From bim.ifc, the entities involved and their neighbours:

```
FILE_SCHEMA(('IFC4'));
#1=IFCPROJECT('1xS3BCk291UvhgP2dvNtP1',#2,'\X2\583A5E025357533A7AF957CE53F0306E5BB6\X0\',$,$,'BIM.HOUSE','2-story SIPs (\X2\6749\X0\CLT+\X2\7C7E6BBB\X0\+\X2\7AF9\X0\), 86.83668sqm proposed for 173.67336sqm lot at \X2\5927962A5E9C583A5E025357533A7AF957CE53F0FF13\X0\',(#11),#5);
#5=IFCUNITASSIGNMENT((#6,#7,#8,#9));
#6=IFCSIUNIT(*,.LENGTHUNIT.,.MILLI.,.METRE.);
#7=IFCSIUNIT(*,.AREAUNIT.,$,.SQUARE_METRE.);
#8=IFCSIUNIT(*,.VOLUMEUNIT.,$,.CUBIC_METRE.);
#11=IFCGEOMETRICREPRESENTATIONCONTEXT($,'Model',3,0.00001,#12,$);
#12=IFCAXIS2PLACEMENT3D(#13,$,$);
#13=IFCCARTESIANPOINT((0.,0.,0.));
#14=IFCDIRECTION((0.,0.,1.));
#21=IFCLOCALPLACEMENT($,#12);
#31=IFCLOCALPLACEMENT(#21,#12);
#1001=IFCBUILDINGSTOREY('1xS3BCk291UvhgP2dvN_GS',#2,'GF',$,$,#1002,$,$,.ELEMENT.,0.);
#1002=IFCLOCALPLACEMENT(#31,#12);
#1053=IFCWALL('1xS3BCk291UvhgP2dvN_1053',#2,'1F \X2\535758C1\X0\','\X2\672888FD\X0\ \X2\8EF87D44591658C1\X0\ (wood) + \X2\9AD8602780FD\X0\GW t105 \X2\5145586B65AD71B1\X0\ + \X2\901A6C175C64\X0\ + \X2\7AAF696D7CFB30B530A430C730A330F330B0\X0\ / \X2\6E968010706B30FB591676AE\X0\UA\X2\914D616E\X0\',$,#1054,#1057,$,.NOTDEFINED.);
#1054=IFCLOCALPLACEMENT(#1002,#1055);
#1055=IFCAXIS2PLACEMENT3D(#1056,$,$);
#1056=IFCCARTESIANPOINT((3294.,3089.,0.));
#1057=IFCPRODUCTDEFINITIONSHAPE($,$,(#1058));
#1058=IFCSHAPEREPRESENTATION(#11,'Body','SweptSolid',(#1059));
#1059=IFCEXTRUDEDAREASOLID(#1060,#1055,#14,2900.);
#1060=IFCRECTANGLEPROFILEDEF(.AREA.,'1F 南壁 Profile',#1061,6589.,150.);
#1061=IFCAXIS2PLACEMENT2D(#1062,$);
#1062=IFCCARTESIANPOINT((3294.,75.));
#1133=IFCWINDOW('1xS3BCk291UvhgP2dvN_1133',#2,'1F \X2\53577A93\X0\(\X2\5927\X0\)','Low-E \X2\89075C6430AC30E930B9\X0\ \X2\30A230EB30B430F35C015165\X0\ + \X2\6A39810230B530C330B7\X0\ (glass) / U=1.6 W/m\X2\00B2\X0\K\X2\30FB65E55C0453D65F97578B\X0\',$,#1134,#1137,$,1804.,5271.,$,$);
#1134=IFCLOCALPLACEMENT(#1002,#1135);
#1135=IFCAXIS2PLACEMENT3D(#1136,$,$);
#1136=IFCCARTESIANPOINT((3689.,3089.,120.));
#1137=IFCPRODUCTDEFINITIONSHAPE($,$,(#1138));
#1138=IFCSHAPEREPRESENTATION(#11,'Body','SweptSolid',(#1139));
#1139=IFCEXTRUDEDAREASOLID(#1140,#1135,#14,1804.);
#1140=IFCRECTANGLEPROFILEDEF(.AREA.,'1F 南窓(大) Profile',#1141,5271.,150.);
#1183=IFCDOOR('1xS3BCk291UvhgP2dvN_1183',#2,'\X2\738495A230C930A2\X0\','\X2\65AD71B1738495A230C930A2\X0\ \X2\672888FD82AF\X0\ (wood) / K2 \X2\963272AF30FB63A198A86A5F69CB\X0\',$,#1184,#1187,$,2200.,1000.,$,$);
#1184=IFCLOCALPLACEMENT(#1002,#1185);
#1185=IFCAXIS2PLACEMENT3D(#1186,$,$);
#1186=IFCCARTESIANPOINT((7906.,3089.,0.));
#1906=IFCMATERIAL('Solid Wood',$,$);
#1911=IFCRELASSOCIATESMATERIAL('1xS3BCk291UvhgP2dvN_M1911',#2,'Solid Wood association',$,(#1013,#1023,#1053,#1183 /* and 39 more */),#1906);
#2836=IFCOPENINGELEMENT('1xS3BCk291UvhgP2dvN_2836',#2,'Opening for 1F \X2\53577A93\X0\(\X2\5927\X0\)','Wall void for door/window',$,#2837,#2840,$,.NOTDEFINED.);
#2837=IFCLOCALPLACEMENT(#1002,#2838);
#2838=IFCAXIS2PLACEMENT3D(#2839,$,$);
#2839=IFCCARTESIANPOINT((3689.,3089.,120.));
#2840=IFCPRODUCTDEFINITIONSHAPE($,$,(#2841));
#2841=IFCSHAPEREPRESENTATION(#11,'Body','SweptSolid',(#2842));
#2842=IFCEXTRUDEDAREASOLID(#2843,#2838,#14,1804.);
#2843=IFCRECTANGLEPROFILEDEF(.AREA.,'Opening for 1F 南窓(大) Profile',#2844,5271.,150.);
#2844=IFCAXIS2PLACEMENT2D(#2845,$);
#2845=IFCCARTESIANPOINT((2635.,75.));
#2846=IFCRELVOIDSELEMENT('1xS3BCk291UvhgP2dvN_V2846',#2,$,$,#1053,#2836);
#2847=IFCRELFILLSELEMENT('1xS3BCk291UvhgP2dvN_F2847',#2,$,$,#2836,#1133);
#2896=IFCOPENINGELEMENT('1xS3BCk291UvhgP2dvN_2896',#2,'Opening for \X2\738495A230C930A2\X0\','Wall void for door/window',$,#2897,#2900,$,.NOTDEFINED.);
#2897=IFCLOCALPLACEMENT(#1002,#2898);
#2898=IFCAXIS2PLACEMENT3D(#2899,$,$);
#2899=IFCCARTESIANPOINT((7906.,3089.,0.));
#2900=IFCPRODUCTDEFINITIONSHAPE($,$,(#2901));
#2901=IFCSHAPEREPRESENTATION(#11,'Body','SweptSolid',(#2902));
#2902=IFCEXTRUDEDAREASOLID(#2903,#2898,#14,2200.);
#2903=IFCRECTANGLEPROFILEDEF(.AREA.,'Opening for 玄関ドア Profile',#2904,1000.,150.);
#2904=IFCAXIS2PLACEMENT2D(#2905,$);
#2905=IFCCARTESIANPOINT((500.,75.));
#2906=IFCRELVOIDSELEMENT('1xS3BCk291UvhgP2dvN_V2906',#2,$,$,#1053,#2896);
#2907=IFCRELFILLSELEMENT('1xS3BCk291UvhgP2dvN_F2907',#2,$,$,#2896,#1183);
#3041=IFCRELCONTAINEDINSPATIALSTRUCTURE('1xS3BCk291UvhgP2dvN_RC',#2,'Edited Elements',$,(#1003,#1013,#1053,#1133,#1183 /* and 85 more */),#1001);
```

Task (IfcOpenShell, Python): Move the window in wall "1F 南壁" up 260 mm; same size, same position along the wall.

```python
import numpy as np
import ifcopenshell
import ifcopenshell.api.geometry
import ifcopenshell.util.placement
import ifcopenshell.util.unit

model = ifcopenshell.open("bim.ifc")
unit_scale = ifcopenshell.util.unit.calculate_unit_scale(model)

window = model.by_id(1133)
opening = window.FillsVoids[0].RelatingOpeningElement
dz = 260.0

shift = np.array([0.0, 0.0, dz])
# The window is not placed relative to its opening, so move both.
for product in (opening, window):
    matrix = ifcopenshell.util.placement.get_local_placement(product.ObjectPlacement)
    matrix[:3, 3] += shift
    ifcopenshell.api.geometry.edit_object_placement(model, product=product, matrix=matrix, is_si=False)

print(f"moved by {dz * unit_scale:+.3f} m")

model.write("bim_v2.ifc")
```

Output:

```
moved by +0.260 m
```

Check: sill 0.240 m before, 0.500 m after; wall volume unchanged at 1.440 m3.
